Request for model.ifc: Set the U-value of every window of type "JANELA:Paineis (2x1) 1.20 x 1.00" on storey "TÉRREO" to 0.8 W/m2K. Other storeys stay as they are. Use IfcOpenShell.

First a look at what the model holds.

```python
import ifcopenshell
import ifcopenshell.util.element

model = ifcopenshell.open("model.ifc")
print(model.schema)
storey = next(s for s in model.by_type("IfcBuildingStorey") if s.Name == "TÉRREO")
windows = [e for e in ifcopenshell.util.element.get_decomposition(storey) if e.is_a("IfcWindow")]
seen = {}
for e in windows:
    element_type = ifcopenshell.util.element.get_type(e)
    key = (element_type.Name if element_type != e and element_type else None, ifcopenshell.util.element.get_pset(e, "Pset_WindowCommon", "ThermalTransmittance"))
    seen[key] = seen.get(key, 0) + 1
for (name, value), count in sorted(seen.items(), key=str):
    print(count, "x", name, "|", value)
```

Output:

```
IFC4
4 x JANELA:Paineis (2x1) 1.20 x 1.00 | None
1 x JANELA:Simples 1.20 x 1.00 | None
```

```python
import ifcopenshell
import ifcopenshell.api.pset
import ifcopenshell.util.element

model = ifcopenshell.open("model.ifc")

storey = next(s for s in model.by_type("IfcBuildingStorey") if s.Name == "TÉRREO")
windows = [e for e in ifcopenshell.util.element.get_decomposition(storey) if e.is_a("IfcWindow")]

count = 0
for e in windows:
    element_type = ifcopenshell.util.element.get_type(e)
    if element_type in (None, e) or element_type.Name != "JANELA:Paineis (2x1) 1.20 x 1.00":
        continue
    # add_pset returns the element's existing set when there is one.
    pset = ifcopenshell.api.pset.add_pset(model, product=e, name="Pset_WindowCommon")
    ifcopenshell.api.pset.edit_pset(model, pset=pset, properties={"ThermalTransmittance": 0.8})
    count += 1

print(count, "windows updated")

model.write("model-out.ifc")
```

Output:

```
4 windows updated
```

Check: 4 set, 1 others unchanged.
